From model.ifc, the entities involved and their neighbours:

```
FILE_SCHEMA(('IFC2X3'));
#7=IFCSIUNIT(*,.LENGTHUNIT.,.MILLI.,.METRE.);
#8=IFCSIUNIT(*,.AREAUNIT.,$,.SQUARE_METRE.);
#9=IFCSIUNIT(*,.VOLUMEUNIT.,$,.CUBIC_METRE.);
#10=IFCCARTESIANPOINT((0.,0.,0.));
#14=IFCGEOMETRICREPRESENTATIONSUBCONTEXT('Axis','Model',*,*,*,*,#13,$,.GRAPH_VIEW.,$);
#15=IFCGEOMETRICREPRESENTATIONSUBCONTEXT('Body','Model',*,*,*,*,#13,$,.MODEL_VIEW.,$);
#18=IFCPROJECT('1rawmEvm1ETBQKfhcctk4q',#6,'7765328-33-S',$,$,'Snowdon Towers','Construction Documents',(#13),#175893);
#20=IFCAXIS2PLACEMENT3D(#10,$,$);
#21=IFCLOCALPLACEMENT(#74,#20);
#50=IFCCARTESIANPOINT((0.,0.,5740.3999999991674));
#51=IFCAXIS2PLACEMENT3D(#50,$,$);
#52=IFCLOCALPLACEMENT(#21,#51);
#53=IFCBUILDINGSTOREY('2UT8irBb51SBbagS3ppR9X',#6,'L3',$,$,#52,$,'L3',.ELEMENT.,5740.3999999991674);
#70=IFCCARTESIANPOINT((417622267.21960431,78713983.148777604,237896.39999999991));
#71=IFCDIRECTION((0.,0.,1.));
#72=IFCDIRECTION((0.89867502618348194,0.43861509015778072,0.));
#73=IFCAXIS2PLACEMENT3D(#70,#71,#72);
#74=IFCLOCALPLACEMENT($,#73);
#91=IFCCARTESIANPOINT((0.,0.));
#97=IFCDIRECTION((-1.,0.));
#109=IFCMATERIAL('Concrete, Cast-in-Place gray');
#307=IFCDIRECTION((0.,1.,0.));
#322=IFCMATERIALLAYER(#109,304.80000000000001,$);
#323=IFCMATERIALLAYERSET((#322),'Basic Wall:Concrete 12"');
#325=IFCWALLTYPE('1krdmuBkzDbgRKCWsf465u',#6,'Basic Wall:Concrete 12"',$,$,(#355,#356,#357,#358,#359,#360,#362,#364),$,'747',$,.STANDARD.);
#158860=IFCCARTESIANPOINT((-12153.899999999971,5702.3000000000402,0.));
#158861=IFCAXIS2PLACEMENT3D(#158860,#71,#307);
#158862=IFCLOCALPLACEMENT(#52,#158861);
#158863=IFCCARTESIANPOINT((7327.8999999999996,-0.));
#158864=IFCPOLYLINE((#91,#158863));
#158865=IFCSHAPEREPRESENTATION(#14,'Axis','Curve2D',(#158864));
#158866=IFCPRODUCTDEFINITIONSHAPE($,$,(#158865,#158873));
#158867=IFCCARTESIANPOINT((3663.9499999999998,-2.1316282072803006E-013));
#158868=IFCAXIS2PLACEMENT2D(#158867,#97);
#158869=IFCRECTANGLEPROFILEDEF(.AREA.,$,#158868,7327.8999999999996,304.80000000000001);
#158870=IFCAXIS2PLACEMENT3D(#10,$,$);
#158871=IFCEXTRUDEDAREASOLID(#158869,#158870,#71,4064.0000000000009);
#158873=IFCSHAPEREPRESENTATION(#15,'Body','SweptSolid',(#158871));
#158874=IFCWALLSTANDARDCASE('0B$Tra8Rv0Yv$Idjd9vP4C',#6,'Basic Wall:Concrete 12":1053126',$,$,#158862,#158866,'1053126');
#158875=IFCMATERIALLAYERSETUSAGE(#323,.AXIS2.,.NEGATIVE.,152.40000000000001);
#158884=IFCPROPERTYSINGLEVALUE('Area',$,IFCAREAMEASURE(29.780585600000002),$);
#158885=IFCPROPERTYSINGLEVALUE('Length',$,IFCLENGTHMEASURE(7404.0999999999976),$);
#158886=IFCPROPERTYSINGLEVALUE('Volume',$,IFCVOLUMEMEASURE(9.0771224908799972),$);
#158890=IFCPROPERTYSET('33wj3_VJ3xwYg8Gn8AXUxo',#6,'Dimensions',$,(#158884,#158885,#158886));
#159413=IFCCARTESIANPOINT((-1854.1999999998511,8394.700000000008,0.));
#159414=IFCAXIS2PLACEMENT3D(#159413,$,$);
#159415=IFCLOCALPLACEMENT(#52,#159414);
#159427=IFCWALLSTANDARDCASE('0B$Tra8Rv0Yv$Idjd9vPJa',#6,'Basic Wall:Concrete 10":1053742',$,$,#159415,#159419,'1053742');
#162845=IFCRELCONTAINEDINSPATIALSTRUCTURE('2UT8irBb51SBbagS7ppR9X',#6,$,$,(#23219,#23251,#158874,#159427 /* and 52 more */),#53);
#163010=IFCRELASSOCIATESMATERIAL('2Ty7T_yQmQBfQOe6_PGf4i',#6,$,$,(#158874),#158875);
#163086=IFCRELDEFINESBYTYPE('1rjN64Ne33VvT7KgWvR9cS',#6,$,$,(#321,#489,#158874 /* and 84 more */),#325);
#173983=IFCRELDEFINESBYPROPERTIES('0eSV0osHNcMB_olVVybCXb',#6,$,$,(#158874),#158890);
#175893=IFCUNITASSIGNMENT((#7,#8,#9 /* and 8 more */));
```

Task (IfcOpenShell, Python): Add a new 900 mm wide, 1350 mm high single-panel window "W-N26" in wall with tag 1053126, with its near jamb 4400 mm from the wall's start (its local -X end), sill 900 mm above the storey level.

```python
import numpy as np
import ifcopenshell
import ifcopenshell.api.feature
import ifcopenshell.api.geometry
import ifcopenshell.api.pset
import ifcopenshell.api.root
import ifcopenshell.api.spatial
import ifcopenshell.api.type
import ifcopenshell.geom
import ifcopenshell.util.element
import ifcopenshell.util.placement
import ifcopenshell.util.representation
import ifcopenshell.util.shape
import ifcopenshell.util.unit

model = ifcopenshell.open("model.ifc")
unit_scale = ifcopenshell.util.unit.calculate_unit_scale(model)
area_scale = ifcopenshell.util.unit.calculate_unit_scale(model, "AREAUNIT")
volume_scale = ifcopenshell.util.unit.calculate_unit_scale(model, "VOLUMEUNIT")
settings = ifcopenshell.geom.settings()


def volume(element):
    """Net volume in cubic metres, openings subtracted."""
    shape = ifcopenshell.geom.create_shape(settings, element)
    return ifcopenshell.util.shape.get_volume(shape.geometry)


wall = model.by_id(158874)
storey = ifcopenshell.util.element.get_container(wall, ifc_class="IfcBuildingStorey")
context = ifcopenshell.util.representation.get_context(model, "Model", "Body", "MODEL_VIEW")
before = volume(wall)

width, height, from_end, sill = 0.9, 1.35, 4.4, 0.9  # metres

# The wall runs along its own X axis, and the end named is its -X end.
wall_shape = ifcopenshell.geom.create_shape(settings, wall)
x, y, z = ifcopenshell.util.shape.get_vertices(wall_shape.geometry).T
start = x.min() + from_end
face, thickness = float(y.min()), float(y.max() - y.min())
wall_matrix = ifcopenshell.util.placement.get_local_placement(wall.ObjectPlacement)
level = ifcopenshell.util.placement.get_local_placement(storey.ObjectPlacement)[2, 3]


def in_wall(x, y):
    """Placement at x, y metres in the wall's axes, at sill height."""
    matrix = wall_matrix.copy()
    matrix[:, 3] = wall_matrix @ np.array([x / unit_scale, y / unit_scale, 0.0, 1.0])
    matrix[2, 3] = level + sill / unit_scale
    return matrix


# Opening: a box that overshoots both wall faces by 50 mm.
opening = ifcopenshell.api.root.create_entity(model, ifc_class="IfcOpeningElement")
box = ifcopenshell.api.geometry.add_wall_representation(
    model, context=context, length=width, height=height, thickness=thickness + 0.1
)
ifcopenshell.api.geometry.assign_representation(model, product=opening, representation=box)
ifcopenshell.api.geometry.edit_object_placement(model, product=opening, matrix=in_wall(start, face - 0.05), is_si=False)
ifcopenshell.api.feature.add_feature(model, feature=opening, element=wall)

window = ifcopenshell.api.root.create_entity(model, ifc_class="IfcWindow", name="W-N26")
window.OverallWidth, window.OverallHeight = width / unit_scale, height / unit_scale
body = ifcopenshell.api.geometry.add_window_representation(
    model,
    context=context,
    overall_width=window.OverallWidth,
    overall_height=window.OverallHeight,
    partition_type="SINGLE_PANEL",
)
ifcopenshell.api.geometry.assign_representation(model, product=window, representation=body)
ifcopenshell.api.spatial.assign_container(model, products=[window], relating_structure=storey)
fills = ifcopenshell.api.feature.add_filling(model, opening=opening, element=window)
fills.OwnerHistory = window.OwnerHistory  # required in IFC2X3

# IFC2X3 keeps the operation on the window style.
style = ifcopenshell.api.root.create_entity(model, ifc_class="IfcWindowStyle", name="W-N26")
style.OperationType, style.ConstructionType = "SINGLE_PANEL", "NOTDEFINED"
style.ParameterTakesPrecedence = style.Sizeable = False
ifcopenshell.api.type.assign_type(model, related_objects=[window], relating_type=style)

# Centre the window in the wall's thickness.
ifcopenshell.api.geometry.edit_object_placement(model, product=window, matrix=in_wall(start, face), is_si=False)
window_shape = ifcopenshell.geom.create_shape(settings, window)
depth = ifcopenshell.util.shape.get_vertices(window_shape.geometry)[:, 1]
offset = face + thickness / 2 - (depth.min() + depth.max()) / 2
ifcopenshell.api.geometry.edit_object_placement(model, product=window, matrix=in_wall(start, offset), is_si=False)

after = volume(wall)

# Update the wall's stored quantities.
pset = model.by_id(ifcopenshell.util.element.get_pset(wall, "Dimensions", should_inherit=False)["id"])
ifcopenshell.api.pset.edit_pset(model, pset=pset, properties={
    "Area": model.create_entity("IfcAreaMeasure", after / thickness / area_scale),
    "Volume": model.create_entity("IfcVolumeMeasure", after / volume_scale),
})

print(f"wall volume {before:.3f} -> {after:.3f} m3")

model.write("model_updated.ifc")
```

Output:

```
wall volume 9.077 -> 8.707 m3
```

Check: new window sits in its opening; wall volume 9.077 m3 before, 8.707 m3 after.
